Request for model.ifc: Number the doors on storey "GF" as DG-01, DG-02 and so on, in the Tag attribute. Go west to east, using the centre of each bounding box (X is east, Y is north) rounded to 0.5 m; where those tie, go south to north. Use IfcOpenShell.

First a look at what the model holds.

```python
import ifcopenshell
import ifcopenshell.util.element
import ifcopenshell.util.placement

model = ifcopenshell.open("model.ifc")
print(model.schema)
storey = next(s for s in model.by_type("IfcBuildingStorey") if s.Name == "GF")
doors = [e for e in ifcopenshell.util.element.get_decomposition(storey) if e.is_a("IfcDoor")]
for e in sorted(doors, key=lambda e: e.id()):
    origin = ifcopenshell.util.placement.get_local_placement(e.ObjectPlacement)[:3, 3]
    print(e.id(), e.Tag, e.Name, origin.round(2) + 0.0, sep=" | ")
```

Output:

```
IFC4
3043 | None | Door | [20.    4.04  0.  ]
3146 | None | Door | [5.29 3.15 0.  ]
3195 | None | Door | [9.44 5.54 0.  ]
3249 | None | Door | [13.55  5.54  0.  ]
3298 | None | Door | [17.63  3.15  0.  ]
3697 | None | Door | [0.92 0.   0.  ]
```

```python
import ifcopenshell
import ifcopenshell.geom
import ifcopenshell.util.element
import ifcopenshell.util.shape

model = ifcopenshell.open("model.ifc")
settings = ifcopenshell.geom.settings()
settings.set("use-world-coords", True)


def centre(element):
    shape = ifcopenshell.geom.create_shape(settings, element)
    return ifcopenshell.util.shape.get_bbox_centroid(shape.geometry)


storey = next(s for s in model.by_type("IfcBuildingStorey") if s.Name == "GF")
doors = [e for e in ifcopenshell.util.element.get_decomposition(storey) if e.is_a("IfcDoor")]

# Insertion points can sit at a corner or the storey origin, so sort by the geometry (in metres).
centres = {e: centre(e) for e in doors}
doors.sort(key=lambda e: (round(centres[e][0] / 0.5), centres[e][1]))

for i, e in enumerate(doors, start=1):
    number = f"DG-{i:02d}"
    e.Tag = number
    print(e.id(), number)

model.write("model_v2.ifc")
```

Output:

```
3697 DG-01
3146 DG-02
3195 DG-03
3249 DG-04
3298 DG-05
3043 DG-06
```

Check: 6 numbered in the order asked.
